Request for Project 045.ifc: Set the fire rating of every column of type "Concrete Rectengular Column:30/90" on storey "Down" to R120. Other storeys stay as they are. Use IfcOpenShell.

First a look at what the model holds.

```python
import ifcopenshell
import ifcopenshell.util.element

model = ifcopenshell.open("Project 045.ifc")
print(model.schema)
storey = next(s for s in model.by_type("IfcBuildingStorey") if s.Name == "Down")
columns = [e for e in ifcopenshell.util.element.get_decomposition(storey) if e.is_a("IfcColumn")]
seen = {}
for e in columns:
    element_type = ifcopenshell.util.element.get_type(e)
    key = (element_type.Name if element_type != e and element_type else None, ifcopenshell.util.element.get_pset(e, "Pset_ColumnCommon", "FireRating"))
    seen[key] = seen.get(key, 0) + 1
for (name, value), count in sorted(seen.items(), key=str):
    print(count, "x", name, "|", value)
```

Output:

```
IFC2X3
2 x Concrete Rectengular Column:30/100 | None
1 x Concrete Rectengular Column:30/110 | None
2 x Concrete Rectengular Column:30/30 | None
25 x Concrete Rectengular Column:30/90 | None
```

```python
import ifcopenshell
import ifcopenshell.api.pset
import ifcopenshell.util.element

model = ifcopenshell.open("Project 045.ifc")

storey = next(s for s in model.by_type("IfcBuildingStorey") if s.Name == "Down")
columns = [e for e in ifcopenshell.util.element.get_decomposition(storey) if e.is_a("IfcColumn")]

count = 0
for e in columns:
    element_type = ifcopenshell.util.element.get_type(e)
    if element_type in (None, e) or element_type.Name != "Concrete Rectengular Column:30/90":
        continue
    # add_pset returns the element's existing set when there is one.
    pset = ifcopenshell.api.pset.add_pset(model, product=e, name="Pset_ColumnCommon")
    ifcopenshell.api.pset.edit_pset(model, pset=pset, properties={"FireRating": "R120"})
    count += 1

print(count, "columns updated")

model.write("Project 045_edited.ifc")
```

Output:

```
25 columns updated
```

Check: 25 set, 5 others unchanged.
